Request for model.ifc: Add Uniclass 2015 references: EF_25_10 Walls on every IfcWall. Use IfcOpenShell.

First a look at what the model holds.

```python
import ifcopenshell

model = ifcopenshell.open("model.ifc")
print(model.schema)
print("classifications:", [c.Name for c in model.by_type("IfcClassification")])
for ifc_class in ("IfcDoor", "IfcRoof", "IfcStair", "IfcWall", "IfcWindow"):
    print(ifc_class, len(model.by_type(ifc_class)))
```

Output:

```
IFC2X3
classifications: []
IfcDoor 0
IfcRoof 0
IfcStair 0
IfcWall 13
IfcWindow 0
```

```python
import ifcopenshell
import ifcopenshell.api.classification

model = ifcopenshell.open("model.ifc")

# IFC2X3 requires Source and Edition and has no link from the project to the system.
system = model.create_entity("IfcClassification", Source="NBS", Edition="2015", Name="Uniclass 2015")

codes = {
    "IfcWall": ("EF_25_10", "Walls"),
}
for ifc_class, (code, name) in codes.items():
    products = model.by_type(ifc_class)
    ifcopenshell.api.classification.add_reference(
        model, products=products, classification=system, identification=code, name=name
    )
    print(code, len(products))

model.write("model_rev.ifc")
```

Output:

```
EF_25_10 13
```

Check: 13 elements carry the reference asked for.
